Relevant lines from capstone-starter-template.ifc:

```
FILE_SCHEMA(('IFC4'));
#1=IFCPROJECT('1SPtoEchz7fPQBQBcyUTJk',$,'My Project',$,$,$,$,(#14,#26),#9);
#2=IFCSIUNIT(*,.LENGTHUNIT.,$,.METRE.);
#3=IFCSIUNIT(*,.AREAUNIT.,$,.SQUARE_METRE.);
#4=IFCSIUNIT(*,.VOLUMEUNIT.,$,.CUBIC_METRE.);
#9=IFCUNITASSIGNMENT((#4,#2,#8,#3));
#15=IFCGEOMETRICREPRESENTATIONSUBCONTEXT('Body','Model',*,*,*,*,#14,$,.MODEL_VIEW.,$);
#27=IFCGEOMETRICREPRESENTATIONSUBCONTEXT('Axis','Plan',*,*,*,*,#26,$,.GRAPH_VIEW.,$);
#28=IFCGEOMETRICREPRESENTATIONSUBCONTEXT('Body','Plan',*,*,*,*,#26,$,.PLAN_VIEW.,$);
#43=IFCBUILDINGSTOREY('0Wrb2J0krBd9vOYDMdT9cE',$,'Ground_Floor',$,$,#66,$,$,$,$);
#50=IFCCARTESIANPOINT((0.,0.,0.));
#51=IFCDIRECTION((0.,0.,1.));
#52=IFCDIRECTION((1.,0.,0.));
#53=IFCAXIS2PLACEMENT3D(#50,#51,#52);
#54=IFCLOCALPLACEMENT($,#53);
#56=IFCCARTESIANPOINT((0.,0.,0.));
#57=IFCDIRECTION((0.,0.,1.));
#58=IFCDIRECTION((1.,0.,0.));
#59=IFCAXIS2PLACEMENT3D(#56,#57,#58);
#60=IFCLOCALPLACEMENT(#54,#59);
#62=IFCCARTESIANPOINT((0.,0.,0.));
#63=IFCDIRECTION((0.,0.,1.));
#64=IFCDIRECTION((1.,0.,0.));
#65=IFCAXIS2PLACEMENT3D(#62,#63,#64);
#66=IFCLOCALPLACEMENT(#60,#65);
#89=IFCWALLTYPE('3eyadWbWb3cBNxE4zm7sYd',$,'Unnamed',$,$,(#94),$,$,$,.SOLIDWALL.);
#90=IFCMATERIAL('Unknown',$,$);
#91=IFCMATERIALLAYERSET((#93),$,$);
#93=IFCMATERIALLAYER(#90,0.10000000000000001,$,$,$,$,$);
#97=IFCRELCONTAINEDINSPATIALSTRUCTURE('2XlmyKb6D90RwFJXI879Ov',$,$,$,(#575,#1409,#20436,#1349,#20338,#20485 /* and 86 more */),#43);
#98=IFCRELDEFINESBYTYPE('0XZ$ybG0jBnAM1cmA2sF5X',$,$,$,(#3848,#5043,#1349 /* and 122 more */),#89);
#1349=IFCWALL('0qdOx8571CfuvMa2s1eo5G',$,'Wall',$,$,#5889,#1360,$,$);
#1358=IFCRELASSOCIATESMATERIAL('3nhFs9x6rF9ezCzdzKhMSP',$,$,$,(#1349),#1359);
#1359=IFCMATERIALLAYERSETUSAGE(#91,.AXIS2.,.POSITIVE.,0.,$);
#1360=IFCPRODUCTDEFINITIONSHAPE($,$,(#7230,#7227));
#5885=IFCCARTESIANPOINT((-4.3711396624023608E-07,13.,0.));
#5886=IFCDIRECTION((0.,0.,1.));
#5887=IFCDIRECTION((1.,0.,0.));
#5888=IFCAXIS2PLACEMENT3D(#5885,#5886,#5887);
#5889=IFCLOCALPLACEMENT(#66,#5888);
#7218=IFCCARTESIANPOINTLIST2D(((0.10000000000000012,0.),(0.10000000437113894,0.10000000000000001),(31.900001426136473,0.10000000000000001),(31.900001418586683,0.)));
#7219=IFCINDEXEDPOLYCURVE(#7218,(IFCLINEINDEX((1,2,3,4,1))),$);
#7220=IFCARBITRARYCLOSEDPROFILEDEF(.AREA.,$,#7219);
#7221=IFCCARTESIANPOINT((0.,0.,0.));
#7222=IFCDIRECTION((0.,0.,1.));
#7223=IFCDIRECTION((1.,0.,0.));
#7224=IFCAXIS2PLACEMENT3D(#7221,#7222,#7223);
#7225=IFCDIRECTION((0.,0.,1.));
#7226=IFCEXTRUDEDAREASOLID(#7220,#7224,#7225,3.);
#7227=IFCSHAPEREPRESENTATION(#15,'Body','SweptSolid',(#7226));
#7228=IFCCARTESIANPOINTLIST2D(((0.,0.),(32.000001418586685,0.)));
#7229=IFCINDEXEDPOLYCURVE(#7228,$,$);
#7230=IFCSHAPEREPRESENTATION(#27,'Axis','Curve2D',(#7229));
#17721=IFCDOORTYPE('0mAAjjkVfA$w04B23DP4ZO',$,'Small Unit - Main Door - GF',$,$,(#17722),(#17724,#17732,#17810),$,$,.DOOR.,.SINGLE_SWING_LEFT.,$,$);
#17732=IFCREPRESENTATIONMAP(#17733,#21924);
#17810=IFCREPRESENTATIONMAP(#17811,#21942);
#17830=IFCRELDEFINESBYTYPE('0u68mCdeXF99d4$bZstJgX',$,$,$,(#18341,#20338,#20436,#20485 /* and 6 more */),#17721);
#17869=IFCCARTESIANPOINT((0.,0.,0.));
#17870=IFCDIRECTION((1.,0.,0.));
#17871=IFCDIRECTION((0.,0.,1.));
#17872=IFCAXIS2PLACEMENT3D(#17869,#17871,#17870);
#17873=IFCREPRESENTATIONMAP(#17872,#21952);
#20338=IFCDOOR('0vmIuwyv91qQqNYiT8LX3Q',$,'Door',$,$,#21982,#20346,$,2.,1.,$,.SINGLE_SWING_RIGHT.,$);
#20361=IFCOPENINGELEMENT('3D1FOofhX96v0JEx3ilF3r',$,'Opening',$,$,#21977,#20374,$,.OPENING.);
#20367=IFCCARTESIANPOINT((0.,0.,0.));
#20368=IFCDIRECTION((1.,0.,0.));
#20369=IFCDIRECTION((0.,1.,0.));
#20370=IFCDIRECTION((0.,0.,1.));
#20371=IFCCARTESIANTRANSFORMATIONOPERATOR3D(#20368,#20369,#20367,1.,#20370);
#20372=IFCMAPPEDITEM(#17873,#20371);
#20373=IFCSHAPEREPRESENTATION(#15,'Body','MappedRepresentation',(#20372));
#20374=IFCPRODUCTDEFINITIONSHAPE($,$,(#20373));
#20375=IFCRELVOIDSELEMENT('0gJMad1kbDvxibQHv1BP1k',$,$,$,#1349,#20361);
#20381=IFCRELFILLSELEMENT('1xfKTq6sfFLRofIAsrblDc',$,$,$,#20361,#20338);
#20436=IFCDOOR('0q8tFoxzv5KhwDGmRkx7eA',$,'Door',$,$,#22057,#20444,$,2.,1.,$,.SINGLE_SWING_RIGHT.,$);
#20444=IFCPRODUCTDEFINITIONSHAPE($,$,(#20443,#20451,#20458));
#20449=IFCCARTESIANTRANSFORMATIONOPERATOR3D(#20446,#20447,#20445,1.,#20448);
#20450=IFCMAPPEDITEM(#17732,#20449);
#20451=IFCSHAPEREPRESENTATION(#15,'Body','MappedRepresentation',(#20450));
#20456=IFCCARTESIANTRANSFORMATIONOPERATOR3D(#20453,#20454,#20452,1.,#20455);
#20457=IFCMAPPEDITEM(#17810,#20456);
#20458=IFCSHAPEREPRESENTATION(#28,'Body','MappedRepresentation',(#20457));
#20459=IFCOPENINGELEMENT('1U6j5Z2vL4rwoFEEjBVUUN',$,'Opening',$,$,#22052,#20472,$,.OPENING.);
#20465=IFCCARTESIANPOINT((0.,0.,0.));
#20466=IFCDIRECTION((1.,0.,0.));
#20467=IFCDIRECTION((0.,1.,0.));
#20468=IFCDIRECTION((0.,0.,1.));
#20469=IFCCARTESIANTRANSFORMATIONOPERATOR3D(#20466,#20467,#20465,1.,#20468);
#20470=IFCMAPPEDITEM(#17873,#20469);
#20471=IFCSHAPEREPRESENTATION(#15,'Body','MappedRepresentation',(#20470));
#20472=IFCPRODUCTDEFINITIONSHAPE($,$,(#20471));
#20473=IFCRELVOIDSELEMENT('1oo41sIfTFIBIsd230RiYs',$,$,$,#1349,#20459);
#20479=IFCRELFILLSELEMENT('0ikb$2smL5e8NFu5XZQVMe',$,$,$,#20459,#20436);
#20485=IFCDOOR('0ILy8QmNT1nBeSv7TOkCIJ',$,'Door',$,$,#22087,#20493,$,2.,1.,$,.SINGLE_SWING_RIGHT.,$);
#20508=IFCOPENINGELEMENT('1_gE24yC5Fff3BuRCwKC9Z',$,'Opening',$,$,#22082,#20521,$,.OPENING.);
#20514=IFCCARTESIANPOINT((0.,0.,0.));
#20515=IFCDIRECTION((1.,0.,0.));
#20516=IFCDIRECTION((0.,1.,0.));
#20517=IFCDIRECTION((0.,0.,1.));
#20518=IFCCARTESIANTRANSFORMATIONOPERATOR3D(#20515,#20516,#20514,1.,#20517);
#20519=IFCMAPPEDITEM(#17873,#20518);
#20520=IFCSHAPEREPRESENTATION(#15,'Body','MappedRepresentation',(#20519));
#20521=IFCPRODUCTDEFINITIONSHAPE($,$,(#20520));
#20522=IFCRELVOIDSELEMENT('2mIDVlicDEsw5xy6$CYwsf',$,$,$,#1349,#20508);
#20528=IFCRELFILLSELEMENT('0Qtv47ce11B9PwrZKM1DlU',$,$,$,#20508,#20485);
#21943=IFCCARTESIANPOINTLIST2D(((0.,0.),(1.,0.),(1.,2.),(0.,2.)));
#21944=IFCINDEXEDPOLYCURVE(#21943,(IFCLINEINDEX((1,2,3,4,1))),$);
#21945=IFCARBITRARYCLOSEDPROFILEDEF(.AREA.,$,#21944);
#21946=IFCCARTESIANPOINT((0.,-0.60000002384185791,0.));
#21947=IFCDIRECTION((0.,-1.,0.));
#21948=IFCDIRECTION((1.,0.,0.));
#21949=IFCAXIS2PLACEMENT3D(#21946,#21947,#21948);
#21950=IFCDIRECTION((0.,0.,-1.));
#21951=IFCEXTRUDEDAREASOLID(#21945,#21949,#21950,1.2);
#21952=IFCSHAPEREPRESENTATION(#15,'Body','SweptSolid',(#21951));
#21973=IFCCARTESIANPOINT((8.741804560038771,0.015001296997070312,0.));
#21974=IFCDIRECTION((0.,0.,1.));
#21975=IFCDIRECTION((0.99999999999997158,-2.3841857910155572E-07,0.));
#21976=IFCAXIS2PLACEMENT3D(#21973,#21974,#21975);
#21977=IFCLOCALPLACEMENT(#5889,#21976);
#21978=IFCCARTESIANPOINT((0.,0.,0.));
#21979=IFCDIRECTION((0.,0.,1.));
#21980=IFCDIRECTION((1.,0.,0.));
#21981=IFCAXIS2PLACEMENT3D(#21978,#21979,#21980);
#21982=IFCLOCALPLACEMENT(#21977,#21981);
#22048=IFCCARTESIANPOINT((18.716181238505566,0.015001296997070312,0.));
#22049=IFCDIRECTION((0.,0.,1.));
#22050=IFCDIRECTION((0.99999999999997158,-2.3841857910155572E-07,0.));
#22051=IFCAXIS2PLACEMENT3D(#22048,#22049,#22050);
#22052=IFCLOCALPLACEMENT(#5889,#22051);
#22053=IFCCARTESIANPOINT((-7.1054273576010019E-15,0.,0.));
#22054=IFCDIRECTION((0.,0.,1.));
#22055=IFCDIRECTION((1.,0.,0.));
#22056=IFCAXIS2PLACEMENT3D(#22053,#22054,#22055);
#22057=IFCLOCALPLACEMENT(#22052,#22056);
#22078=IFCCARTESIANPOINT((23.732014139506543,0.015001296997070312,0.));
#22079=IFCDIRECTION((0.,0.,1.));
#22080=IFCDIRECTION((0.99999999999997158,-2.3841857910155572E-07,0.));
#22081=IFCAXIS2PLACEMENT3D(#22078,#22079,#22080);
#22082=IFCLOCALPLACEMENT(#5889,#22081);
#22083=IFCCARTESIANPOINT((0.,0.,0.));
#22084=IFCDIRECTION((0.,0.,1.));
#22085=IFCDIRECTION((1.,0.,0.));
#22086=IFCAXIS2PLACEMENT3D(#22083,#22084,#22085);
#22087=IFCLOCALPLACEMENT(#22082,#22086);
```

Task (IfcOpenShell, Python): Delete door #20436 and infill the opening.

```python
import ifcopenshell
import ifcopenshell.api.feature
import ifcopenshell.api.root
import ifcopenshell.geom
import ifcopenshell.util.shape

model = ifcopenshell.open("capstone-starter-template.ifc")
settings = ifcopenshell.geom.settings()


def volume(element):
    """Net volume in cubic metres, openings subtracted."""
    shape = ifcopenshell.geom.create_shape(settings, element)
    return ifcopenshell.util.shape.get_volume(shape.geometry)


door = model.by_guid("0q8tFoxzv5KhwDGmRkx7eA")
opening = door.FillsVoids[0].RelatingOpeningElement
wall = opening.VoidsElements[0].RelatingBuildingElement
before = volume(wall)

ifcopenshell.api.root.remove_product(model, product=door)
ifcopenshell.api.feature.remove_feature(model, feature=opening)

after = volume(wall)

print(f"wall volume {before:.3f} -> {after:.3f} m3")

model.write("capstone-starter-template_rev.ifc")
```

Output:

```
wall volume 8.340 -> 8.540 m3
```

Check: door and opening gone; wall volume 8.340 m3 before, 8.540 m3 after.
